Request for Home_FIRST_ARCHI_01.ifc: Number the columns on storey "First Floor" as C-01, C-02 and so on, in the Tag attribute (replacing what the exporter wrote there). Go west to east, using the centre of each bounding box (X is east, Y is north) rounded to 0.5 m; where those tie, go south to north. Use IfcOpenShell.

First a look at what the model holds.

```python
import ifcopenshell
import ifcopenshell.util.element
import ifcopenshell.util.placement

model = ifcopenshell.open("Home_FIRST_ARCHI_01.ifc")
print(model.schema)
storey = next(s for s in model.by_type("IfcBuildingStorey") if s.Name == "First Floor")
columns = [e for e in ifcopenshell.util.element.get_decomposition(storey) if e.is_a("IfcColumn")]
for e in sorted(columns, key=lambda e: e.id()):
    origin = ifcopenshell.util.placement.get_local_placement(e.ObjectPlacement)[:3, 3]
    print(e.id(), e.Tag, e.Name, origin.round(2) + 0.0, sep=" | ")
```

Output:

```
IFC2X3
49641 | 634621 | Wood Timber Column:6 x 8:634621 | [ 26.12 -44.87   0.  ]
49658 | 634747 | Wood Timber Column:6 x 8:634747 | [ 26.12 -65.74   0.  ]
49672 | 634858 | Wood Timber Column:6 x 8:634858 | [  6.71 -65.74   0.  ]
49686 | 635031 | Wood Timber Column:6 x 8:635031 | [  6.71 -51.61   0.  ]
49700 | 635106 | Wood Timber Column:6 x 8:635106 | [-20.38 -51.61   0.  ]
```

```python
import ifcopenshell
import ifcopenshell.geom
import ifcopenshell.util.element
import ifcopenshell.util.shape

model = ifcopenshell.open("Home_FIRST_ARCHI_01.ifc")
settings = ifcopenshell.geom.settings()
settings.set("use-world-coords", True)


def centre(element):
    shape = ifcopenshell.geom.create_shape(settings, element)
    return ifcopenshell.util.shape.get_bbox_centroid(shape.geometry)


storey = next(s for s in model.by_type("IfcBuildingStorey") if s.Name == "First Floor")
columns = [e for e in ifcopenshell.util.element.get_decomposition(storey) if e.is_a("IfcColumn")]

# Insertion points can sit at a corner or the storey origin, so sort by the geometry (in metres).
centres = {e: centre(e) for e in columns}
columns.sort(key=lambda e: (round(centres[e][0] / 0.5), centres[e][1]))

for i, e in enumerate(columns, start=1):
    number = f"C-{i:02d}"
    e.Tag = number
    print(e.id(), number)

model.write("Home_FIRST_ARCHI_01_updated.ifc")
```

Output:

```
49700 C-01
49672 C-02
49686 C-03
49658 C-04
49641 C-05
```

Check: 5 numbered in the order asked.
